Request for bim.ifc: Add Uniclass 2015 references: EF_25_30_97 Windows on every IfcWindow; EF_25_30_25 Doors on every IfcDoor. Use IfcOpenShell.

First a look at what the model holds.

```python
import ifcopenshell

model = ifcopenshell.open("bim.ifc")
print(model.schema)
print("classifications:", [c.Name for c in model.by_type("IfcClassification")])
for ifc_class in ("IfcDoor", "IfcRoof", "IfcStair", "IfcWall", "IfcWindow"):
    print(ifc_class, len(model.by_type(ifc_class)))
```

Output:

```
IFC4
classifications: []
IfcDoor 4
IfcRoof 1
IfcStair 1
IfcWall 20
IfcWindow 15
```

```python
import ifcopenshell
import ifcopenshell.api.classification

model = ifcopenshell.open("bim.ifc")

system = ifcopenshell.api.classification.add_classification(model, classification="Uniclass 2015")

codes = {
    "IfcWindow": ("EF_25_30_97", "Windows"),
    "IfcDoor": ("EF_25_30_25", "Doors"),
}
for ifc_class, (code, name) in codes.items():
    products = model.by_type(ifc_class)
    ifcopenshell.api.classification.add_reference(
        model, products=products, classification=system, identification=code, name=name
    )
    print(code, len(products))

model.write("bim_edited.ifc")
```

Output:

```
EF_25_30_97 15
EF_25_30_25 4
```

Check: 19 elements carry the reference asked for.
